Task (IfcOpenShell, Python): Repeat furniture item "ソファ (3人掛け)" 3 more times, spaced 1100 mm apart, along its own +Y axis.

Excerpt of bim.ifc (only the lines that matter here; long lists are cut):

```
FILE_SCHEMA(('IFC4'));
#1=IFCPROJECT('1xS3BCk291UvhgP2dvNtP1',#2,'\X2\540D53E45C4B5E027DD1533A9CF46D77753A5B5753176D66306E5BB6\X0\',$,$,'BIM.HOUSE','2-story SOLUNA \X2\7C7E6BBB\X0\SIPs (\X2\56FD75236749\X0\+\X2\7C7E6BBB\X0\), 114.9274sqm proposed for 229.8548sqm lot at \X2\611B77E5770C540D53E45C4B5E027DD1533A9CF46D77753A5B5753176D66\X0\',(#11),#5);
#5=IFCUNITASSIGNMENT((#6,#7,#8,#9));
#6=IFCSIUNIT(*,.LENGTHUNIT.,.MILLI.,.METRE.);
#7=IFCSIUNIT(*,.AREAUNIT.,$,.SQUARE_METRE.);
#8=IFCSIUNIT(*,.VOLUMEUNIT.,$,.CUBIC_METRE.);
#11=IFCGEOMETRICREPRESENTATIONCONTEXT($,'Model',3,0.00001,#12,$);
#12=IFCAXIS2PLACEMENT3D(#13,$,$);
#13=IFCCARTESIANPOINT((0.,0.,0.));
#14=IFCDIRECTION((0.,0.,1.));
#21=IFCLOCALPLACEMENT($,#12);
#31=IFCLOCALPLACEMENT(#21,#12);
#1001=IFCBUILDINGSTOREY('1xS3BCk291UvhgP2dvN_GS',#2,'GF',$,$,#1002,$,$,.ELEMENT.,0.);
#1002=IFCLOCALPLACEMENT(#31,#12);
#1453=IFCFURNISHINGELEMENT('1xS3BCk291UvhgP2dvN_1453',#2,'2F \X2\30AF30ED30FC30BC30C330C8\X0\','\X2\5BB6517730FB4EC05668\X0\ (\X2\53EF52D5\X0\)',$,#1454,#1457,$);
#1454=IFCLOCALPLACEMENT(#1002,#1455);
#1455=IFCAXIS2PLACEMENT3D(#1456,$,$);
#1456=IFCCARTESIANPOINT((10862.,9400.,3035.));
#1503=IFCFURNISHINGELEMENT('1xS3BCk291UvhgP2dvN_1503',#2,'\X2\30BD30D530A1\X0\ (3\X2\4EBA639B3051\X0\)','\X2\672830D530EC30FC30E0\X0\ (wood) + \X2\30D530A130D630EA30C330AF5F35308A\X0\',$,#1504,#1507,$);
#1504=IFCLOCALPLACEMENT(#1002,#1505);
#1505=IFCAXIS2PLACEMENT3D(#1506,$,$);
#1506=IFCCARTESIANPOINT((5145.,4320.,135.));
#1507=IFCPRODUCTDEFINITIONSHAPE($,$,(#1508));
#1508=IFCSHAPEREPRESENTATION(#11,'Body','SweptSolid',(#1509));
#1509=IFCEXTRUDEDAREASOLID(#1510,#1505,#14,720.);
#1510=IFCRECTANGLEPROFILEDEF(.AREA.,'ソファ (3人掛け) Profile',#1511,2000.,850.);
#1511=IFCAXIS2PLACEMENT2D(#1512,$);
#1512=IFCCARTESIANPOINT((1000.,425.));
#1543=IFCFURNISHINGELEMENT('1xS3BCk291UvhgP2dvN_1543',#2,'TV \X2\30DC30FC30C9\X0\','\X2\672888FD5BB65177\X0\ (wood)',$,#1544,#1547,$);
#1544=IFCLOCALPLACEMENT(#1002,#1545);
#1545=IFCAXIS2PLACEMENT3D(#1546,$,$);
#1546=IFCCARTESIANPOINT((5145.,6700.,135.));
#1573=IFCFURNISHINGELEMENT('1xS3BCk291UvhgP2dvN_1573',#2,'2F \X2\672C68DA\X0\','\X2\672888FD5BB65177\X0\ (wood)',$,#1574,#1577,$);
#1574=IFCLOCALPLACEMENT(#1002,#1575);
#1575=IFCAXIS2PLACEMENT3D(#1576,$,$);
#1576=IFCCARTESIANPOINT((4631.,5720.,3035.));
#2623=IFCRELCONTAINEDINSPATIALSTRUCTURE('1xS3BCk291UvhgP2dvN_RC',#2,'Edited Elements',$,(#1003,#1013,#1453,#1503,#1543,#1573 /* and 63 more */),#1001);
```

```python
import ifcopenshell
import ifcopenshell.api.geometry
import ifcopenshell.api.root
import ifcopenshell.util.element
import ifcopenshell.util.placement
import ifcopenshell.util.unit

model = ifcopenshell.open("bim.ifc")
unit_scale = ifcopenshell.util.unit.calculate_unit_scale(model)


def reuse_history(source, copy):
    """copy_class also copies each property set's owner history, people and application; keep the originals."""
    for rel in copy.IsDefinedBy:
        if rel.is_a("IfcRelDefinesByProperties") and (history := rel.RelatingPropertyDefinition.OwnerHistory):
            rel.RelatingPropertyDefinition.OwnerHistory = source.OwnerHistory
            ifcopenshell.util.element.remove_deep2(model, history)


source = model.by_guid("1xS3BCk291UvhgP2dvN_1503")
base = ifcopenshell.util.placement.get_local_placement(source.ObjectPlacement)
step = base[:3, 1] * 1.1 / unit_scale

for i in range(1, 4):
    copy = ifcopenshell.api.root.copy_class(model, product=source)
    copy.Representation = ifcopenshell.util.element.copy_deep(
        model, source.Representation, exclude=["IfcGeometricRepresentationContext", "IfcRepresentationMap"]
    )
    reuse_history(source, copy)
    matrix = base.copy()
    matrix[:3, 3] += i * step
    print("added at", matrix[:3, 3].round(3) + 0.0)
    ifcopenshell.api.geometry.edit_object_placement(model, product=copy, matrix=matrix, is_si=False)

model.write("bim_updated.ifc")
```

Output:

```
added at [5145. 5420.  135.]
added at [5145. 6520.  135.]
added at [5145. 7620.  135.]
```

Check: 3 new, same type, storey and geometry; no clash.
